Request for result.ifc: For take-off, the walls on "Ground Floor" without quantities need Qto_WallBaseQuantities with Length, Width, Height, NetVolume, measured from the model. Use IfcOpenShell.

First a look at what the model holds.

```python
import ifcopenshell
import ifcopenshell.util.element
import ifcopenshell.util.unit

model = ifcopenshell.open("result.ifc")
print(model.schema)
for unit_type in ("LENGTHUNIT", "AREAUNIT", "VOLUMEUNIT"):
    print(unit_type, ifcopenshell.util.unit.calculate_unit_scale(model, unit_type))
storey = next(s for s in model.by_type("IfcBuildingStorey") if s.Name == "Ground Floor")
walls = [e for e in ifcopenshell.util.element.get_decomposition(storey) if e.is_a("IfcWall")]
for e in sorted(walls, key=lambda e: e.id()):
    print(e.id(), e.is_a(), e.Name, list(ifcopenshell.util.element.get_psets(e, qtos_only=True)), sep=" | ")
```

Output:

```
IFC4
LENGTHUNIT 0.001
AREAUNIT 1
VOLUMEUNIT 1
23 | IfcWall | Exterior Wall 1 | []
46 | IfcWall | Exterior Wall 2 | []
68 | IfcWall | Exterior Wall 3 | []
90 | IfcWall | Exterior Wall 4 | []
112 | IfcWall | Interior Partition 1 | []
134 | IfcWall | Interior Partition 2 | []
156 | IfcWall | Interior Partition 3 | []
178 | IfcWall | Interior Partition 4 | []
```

```python
import ifcopenshell
import ifcopenshell.api.pset
import ifcopenshell.geom
import ifcopenshell.util.element
import ifcopenshell.util.shape
import ifcopenshell.util.unit

model = ifcopenshell.open("result.ifc")
unit_scale = ifcopenshell.util.unit.calculate_unit_scale(model)
volume_scale = ifcopenshell.util.unit.calculate_unit_scale(model, "VOLUMEUNIT")
settings = ifcopenshell.geom.settings()

storey = next(s for s in model.by_type("IfcBuildingStorey") if s.Name == "Ground Floor")
walls = [e for e in ifcopenshell.util.element.get_decomposition(storey) if e.is_a("IfcWall")]

for e in sorted(walls, key=lambda e: e.id()):
    if ifcopenshell.util.element.get_psets(e, qtos_only=True, should_inherit=False):
        continue
    # Geometry comes back in metres, in the element's own axes.
    shape = ifcopenshell.geom.create_shape(settings, e)
    values = {
        "Length": ifcopenshell.util.shape.get_x(shape.geometry) / unit_scale,
        "Width": ifcopenshell.util.shape.get_y(shape.geometry) / unit_scale,
        "Height": ifcopenshell.util.shape.get_z(shape.geometry) / unit_scale,
        "NetVolume": ifcopenshell.util.shape.get_volume(shape.geometry) / volume_scale,
    }
    qto = ifcopenshell.api.pset.add_qto(model, product=e, name="Qto_WallBaseQuantities")
    ifcopenshell.api.pset.edit_qto(model, qto=qto, properties=values)
    print(e.id(), {k: round(v, 3) for k, v in values.items()})

model.write("result-out.ifc")
```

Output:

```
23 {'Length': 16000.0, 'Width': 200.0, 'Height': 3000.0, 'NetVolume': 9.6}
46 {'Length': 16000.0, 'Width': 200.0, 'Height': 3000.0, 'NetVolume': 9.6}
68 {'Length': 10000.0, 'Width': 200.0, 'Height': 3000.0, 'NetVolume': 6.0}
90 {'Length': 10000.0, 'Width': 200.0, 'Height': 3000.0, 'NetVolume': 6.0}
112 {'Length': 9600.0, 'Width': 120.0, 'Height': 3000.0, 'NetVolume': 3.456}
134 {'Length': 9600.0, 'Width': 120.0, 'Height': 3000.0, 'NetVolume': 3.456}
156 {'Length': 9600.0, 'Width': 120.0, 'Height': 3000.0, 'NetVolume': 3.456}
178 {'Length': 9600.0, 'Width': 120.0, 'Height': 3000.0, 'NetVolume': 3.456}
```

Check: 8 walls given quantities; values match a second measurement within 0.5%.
